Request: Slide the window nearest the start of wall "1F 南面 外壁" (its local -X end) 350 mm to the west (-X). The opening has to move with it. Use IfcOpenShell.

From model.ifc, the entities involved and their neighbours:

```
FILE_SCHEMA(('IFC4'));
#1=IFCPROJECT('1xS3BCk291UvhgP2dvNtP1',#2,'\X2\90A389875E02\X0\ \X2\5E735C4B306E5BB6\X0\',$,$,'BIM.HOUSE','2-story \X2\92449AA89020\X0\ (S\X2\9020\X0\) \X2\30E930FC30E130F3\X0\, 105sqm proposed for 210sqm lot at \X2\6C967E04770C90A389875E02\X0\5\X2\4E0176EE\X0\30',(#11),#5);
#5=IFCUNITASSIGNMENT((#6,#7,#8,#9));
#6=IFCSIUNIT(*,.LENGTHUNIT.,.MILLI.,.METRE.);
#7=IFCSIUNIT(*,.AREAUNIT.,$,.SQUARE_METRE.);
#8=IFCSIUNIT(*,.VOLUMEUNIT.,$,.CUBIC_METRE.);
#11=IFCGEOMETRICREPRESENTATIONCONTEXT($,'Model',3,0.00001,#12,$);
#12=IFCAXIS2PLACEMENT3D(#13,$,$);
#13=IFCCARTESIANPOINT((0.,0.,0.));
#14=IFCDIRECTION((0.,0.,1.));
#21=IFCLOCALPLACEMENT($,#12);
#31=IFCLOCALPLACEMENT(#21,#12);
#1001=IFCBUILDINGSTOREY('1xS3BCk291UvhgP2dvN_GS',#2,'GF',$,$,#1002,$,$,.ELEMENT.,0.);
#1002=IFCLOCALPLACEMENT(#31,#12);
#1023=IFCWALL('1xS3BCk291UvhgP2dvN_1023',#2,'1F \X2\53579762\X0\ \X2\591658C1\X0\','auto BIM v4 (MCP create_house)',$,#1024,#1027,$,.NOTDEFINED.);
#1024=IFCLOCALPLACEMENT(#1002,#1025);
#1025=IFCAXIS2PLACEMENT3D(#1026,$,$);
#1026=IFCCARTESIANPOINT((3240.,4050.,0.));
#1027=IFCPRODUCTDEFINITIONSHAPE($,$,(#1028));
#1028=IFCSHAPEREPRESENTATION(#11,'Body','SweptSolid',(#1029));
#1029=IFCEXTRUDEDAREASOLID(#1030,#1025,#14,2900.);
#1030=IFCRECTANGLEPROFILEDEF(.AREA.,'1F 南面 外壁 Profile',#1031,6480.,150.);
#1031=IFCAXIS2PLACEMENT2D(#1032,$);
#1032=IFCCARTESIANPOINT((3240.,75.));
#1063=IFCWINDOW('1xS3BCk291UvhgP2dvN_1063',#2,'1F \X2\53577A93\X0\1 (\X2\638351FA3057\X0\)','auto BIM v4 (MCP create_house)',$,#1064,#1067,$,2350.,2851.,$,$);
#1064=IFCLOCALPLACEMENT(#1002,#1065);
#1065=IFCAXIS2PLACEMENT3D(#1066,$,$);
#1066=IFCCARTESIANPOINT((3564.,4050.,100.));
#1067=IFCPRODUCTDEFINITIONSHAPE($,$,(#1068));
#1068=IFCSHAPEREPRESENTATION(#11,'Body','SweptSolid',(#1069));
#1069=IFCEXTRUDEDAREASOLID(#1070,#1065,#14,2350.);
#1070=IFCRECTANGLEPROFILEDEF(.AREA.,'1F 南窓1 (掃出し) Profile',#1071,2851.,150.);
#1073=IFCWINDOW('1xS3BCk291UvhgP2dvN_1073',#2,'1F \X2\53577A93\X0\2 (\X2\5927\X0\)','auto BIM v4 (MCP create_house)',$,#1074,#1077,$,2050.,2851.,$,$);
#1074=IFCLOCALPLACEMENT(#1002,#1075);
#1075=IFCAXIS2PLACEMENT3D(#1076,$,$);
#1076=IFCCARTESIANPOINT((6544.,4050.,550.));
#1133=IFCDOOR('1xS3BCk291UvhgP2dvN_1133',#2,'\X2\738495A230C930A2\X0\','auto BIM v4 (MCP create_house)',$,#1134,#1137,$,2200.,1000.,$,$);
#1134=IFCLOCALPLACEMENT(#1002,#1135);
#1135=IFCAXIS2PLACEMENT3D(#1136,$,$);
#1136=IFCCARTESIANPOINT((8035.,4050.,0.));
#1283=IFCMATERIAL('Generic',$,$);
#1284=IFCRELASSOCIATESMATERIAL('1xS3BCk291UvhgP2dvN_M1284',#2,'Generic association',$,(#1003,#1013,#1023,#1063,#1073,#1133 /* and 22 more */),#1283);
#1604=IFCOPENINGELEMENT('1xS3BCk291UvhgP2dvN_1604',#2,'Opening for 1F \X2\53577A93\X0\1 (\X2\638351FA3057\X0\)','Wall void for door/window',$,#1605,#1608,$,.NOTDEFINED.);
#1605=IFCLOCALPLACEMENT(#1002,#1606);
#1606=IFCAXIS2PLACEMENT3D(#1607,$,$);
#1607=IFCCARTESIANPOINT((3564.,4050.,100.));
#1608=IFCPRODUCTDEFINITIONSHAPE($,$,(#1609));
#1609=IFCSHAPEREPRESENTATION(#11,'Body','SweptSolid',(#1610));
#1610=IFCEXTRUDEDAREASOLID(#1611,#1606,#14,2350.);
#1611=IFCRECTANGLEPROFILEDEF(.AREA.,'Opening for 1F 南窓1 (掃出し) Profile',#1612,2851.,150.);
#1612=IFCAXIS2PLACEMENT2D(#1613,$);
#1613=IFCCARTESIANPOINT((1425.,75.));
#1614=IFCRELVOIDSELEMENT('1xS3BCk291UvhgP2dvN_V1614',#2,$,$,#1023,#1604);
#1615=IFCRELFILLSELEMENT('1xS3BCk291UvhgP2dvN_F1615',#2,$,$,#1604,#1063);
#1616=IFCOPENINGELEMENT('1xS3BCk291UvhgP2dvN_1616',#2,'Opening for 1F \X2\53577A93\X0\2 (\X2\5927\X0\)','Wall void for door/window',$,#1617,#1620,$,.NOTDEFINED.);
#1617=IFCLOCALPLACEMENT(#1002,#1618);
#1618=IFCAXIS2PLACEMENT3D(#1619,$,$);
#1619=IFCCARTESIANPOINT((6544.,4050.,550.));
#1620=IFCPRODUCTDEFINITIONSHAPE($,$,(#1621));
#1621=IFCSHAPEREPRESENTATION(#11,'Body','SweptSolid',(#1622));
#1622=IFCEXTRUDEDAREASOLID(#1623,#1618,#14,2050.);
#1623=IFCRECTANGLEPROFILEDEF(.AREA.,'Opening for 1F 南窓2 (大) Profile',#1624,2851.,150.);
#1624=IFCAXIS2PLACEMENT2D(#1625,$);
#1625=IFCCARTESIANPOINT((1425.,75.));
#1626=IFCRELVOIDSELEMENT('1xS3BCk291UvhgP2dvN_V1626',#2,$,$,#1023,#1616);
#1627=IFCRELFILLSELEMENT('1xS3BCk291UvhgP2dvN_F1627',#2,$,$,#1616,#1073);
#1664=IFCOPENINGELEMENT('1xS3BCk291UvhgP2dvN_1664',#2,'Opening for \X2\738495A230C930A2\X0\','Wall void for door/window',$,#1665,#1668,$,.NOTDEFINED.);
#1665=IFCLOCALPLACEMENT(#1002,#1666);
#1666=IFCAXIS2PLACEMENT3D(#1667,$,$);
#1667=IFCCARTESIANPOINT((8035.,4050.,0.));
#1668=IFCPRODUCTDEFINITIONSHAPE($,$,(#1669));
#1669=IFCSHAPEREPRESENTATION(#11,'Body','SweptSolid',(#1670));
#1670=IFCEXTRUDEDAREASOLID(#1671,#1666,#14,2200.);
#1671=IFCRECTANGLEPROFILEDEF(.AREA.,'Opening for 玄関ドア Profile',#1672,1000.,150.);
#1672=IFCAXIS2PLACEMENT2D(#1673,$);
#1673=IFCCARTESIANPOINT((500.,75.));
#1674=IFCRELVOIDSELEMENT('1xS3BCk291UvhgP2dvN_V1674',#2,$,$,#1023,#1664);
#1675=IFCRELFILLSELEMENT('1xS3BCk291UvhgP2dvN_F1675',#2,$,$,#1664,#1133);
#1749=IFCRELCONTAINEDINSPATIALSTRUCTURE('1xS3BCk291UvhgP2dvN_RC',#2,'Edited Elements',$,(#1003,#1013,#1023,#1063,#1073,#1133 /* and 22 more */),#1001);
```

```python
import ifcopenshell
import ifcopenshell.api.geometry
import ifcopenshell.util.placement
import ifcopenshell.util.unit

model = ifcopenshell.open("model.ifc")
unit_scale = ifcopenshell.util.unit.calculate_unit_scale(model)

window = model.by_guid("1xS3BCk291UvhgP2dvN_1063")
opening = window.FillsVoids[0].RelatingOpeningElement
wall = opening.VoidsElements[0].RelatingBuildingElement

wall_matrix = ifcopenshell.util.placement.get_local_placement(wall.ObjectPlacement)
shift = wall_matrix[:3, 0] * -0.35 / unit_scale
before = ifcopenshell.util.placement.get_local_placement(window.ObjectPlacement)[:3, 3].copy()

# The window is not placed relative to its opening, so move both.
for product in (opening, window):
    matrix = ifcopenshell.util.placement.get_local_placement(product.ObjectPlacement)
    matrix[:3, 3] += shift
    ifcopenshell.api.geometry.edit_object_placement(model, product=product, matrix=matrix, is_si=False)

after = ifcopenshell.util.placement.get_local_placement(window.ObjectPlacement)[:3, 3]
print("window moved by", (after - before).round(3) + 0.0)

model.write("model_rev.ifc")
```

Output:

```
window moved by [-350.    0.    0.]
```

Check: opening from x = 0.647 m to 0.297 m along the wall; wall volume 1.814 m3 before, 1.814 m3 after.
